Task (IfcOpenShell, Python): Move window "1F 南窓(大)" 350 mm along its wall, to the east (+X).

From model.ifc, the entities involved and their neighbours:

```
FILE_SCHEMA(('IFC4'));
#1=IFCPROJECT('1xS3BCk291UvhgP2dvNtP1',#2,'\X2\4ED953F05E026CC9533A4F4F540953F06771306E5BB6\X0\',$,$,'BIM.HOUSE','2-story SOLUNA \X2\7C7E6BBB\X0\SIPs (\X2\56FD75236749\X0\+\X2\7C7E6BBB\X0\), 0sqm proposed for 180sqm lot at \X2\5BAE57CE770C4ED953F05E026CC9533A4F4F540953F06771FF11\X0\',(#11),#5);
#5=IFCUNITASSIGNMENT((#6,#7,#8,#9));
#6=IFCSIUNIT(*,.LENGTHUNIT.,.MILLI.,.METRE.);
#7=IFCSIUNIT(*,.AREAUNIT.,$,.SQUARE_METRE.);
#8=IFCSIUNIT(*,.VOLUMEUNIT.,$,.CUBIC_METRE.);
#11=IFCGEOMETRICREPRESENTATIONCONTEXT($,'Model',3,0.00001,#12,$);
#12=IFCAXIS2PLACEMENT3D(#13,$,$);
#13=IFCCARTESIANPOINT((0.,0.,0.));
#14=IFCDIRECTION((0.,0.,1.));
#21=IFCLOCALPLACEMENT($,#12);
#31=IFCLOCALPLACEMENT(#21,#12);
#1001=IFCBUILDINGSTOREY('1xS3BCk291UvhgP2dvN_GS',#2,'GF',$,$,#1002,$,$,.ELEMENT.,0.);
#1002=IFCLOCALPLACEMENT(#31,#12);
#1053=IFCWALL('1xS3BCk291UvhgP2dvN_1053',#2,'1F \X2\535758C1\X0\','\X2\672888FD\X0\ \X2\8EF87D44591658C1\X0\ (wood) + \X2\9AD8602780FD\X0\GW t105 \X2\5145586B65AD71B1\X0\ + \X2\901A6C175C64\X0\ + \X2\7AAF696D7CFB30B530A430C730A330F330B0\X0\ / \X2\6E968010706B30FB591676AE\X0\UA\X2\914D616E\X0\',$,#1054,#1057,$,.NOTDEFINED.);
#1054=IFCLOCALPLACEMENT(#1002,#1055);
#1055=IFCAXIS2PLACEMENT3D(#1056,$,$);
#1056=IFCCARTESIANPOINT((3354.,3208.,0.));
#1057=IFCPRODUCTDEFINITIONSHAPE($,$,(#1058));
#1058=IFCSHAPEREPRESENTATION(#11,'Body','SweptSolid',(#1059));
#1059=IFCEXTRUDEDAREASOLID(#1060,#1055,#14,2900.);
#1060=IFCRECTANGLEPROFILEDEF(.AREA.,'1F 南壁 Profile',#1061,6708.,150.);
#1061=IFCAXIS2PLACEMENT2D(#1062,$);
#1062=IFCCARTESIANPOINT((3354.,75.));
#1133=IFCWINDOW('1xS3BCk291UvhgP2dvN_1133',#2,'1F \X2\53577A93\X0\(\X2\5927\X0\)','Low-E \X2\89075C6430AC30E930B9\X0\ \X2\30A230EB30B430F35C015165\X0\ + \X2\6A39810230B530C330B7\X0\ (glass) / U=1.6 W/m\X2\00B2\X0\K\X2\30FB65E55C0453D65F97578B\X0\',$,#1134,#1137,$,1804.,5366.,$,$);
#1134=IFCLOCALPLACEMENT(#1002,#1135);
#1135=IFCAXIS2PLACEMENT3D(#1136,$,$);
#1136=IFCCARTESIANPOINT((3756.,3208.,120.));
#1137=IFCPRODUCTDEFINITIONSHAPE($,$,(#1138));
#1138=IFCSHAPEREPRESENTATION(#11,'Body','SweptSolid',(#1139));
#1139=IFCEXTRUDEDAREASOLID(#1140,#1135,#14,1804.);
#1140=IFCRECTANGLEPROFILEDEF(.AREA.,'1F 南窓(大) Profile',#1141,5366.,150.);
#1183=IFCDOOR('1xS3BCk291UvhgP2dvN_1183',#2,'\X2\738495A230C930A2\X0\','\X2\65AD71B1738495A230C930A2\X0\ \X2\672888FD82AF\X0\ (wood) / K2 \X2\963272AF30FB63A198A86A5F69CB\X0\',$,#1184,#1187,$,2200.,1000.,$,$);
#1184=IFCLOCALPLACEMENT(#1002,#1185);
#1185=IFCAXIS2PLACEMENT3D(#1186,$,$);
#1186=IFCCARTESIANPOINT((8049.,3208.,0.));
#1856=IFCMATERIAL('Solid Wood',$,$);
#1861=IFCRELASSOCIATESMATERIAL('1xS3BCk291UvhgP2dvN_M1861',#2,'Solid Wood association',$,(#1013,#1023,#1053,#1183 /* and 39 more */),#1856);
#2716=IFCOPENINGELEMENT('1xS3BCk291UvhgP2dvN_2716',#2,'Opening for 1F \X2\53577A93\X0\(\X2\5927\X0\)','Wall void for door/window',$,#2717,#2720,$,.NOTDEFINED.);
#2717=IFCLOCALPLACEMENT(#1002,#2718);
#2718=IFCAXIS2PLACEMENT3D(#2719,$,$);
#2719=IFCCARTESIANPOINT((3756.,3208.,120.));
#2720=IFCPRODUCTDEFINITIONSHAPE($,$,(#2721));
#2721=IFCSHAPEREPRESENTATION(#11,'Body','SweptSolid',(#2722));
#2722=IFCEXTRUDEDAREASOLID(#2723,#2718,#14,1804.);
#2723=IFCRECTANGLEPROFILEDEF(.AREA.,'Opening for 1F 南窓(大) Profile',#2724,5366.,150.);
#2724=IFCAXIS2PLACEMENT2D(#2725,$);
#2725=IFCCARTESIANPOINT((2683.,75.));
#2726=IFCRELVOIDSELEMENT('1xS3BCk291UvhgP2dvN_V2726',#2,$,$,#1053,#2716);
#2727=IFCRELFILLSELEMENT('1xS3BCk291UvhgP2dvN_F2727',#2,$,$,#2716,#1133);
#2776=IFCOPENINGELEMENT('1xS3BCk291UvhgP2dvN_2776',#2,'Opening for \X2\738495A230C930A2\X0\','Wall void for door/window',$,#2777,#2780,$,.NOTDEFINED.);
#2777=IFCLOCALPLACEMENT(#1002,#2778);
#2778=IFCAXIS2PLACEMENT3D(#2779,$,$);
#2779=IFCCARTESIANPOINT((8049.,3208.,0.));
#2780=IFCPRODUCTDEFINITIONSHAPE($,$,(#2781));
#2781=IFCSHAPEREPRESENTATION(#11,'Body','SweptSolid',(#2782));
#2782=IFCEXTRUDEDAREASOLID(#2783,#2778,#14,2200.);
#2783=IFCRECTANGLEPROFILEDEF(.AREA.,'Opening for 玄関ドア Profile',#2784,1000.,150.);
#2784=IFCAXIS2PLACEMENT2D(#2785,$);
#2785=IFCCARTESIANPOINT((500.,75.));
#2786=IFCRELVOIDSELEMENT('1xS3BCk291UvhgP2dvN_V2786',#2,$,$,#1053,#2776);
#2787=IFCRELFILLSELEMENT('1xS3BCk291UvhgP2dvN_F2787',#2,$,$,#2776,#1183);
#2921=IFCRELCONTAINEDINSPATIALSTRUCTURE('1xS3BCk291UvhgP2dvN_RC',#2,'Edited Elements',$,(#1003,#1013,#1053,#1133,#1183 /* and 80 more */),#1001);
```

```python
import ifcopenshell
import ifcopenshell.api.geometry
import ifcopenshell.util.placement
import ifcopenshell.util.unit

model = ifcopenshell.open("model.ifc")
unit_scale = ifcopenshell.util.unit.calculate_unit_scale(model)

window = model.by_guid("1xS3BCk291UvhgP2dvN_1133")
opening = window.FillsVoids[0].RelatingOpeningElement
wall = opening.VoidsElements[0].RelatingBuildingElement

wall_matrix = ifcopenshell.util.placement.get_local_placement(wall.ObjectPlacement)
shift = wall_matrix[:3, 0] * 0.35 / unit_scale
before = ifcopenshell.util.placement.get_local_placement(window.ObjectPlacement)[:3, 3].copy()

# The window is not placed relative to its opening, so move both.
for product in (opening, window):
    matrix = ifcopenshell.util.placement.get_local_placement(product.ObjectPlacement)
    matrix[:3, 3] += shift
    ifcopenshell.api.geometry.edit_object_placement(model, product=product, matrix=matrix, is_si=False)

after = ifcopenshell.util.placement.get_local_placement(window.ObjectPlacement)[:3, 3]
print("window moved by", (after - before).round(3) + 0.0)

model.write("model_v2.ifc")
```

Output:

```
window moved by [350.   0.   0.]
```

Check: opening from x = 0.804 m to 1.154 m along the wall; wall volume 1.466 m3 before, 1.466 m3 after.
